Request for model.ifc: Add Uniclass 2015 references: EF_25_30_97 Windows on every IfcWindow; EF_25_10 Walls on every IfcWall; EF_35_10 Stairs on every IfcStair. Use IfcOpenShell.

First a look at what the model holds.

```python
import ifcopenshell

model = ifcopenshell.open("model.ifc")
print(model.schema)
print("classifications:", [c.Name for c in model.by_type("IfcClassification")])
for ifc_class in ("IfcDoor", "IfcRoof", "IfcStair", "IfcWall", "IfcWindow"):
    print(ifc_class, len(model.by_type(ifc_class)))
```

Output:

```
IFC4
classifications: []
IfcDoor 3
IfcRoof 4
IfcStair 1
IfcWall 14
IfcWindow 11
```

```python
import ifcopenshell
import ifcopenshell.api.classification

model = ifcopenshell.open("model.ifc")

system = ifcopenshell.api.classification.add_classification(model, classification="Uniclass 2015")

codes = {
    "IfcWindow": ("EF_25_30_97", "Windows"),
    "IfcWall": ("EF_25_10", "Walls"),
    "IfcStair": ("EF_35_10", "Stairs"),
}
for ifc_class, (code, name) in codes.items():
    products = model.by_type(ifc_class)
    ifcopenshell.api.classification.add_reference(
        model, products=products, classification=system, identification=code, name=name
    )
    print(code, len(products))

model.write("model_updated.ifc")
```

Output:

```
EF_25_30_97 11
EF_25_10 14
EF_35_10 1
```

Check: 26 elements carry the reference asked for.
